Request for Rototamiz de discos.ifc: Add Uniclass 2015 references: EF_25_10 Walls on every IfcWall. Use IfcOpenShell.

First a look at what the model holds.

```python
import ifcopenshell

model = ifcopenshell.open("Rototamiz de discos.ifc")
print(model.schema)
print("classifications:", [c.Name for c in model.by_type("IfcClassification")])
for ifc_class in ("IfcDoor", "IfcRoof", "IfcStair", "IfcWall", "IfcWindow"):
    print(ifc_class, len(model.by_type(ifc_class)))
```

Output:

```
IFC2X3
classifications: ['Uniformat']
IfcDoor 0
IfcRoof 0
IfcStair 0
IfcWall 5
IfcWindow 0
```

```python
import ifcopenshell
import ifcopenshell.api.classification

model = ifcopenshell.open("Rototamiz de discos.ifc")

# IFC2X3 requires Source and Edition and has no link from the project to the system.
system = model.create_entity("IfcClassification", Source="NBS", Edition="2015", Name="Uniclass 2015")

codes = {
    "IfcWall": ("EF_25_10", "Walls"),
}
for ifc_class, (code, name) in codes.items():
    products = model.by_type(ifc_class)
    ifcopenshell.api.classification.add_reference(
        model, products=products, classification=system, identification=code, name=name
    )
    print(code, len(products))

model.write("Rototamiz de discos_edited.ifc")
```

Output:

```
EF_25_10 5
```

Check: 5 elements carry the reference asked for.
